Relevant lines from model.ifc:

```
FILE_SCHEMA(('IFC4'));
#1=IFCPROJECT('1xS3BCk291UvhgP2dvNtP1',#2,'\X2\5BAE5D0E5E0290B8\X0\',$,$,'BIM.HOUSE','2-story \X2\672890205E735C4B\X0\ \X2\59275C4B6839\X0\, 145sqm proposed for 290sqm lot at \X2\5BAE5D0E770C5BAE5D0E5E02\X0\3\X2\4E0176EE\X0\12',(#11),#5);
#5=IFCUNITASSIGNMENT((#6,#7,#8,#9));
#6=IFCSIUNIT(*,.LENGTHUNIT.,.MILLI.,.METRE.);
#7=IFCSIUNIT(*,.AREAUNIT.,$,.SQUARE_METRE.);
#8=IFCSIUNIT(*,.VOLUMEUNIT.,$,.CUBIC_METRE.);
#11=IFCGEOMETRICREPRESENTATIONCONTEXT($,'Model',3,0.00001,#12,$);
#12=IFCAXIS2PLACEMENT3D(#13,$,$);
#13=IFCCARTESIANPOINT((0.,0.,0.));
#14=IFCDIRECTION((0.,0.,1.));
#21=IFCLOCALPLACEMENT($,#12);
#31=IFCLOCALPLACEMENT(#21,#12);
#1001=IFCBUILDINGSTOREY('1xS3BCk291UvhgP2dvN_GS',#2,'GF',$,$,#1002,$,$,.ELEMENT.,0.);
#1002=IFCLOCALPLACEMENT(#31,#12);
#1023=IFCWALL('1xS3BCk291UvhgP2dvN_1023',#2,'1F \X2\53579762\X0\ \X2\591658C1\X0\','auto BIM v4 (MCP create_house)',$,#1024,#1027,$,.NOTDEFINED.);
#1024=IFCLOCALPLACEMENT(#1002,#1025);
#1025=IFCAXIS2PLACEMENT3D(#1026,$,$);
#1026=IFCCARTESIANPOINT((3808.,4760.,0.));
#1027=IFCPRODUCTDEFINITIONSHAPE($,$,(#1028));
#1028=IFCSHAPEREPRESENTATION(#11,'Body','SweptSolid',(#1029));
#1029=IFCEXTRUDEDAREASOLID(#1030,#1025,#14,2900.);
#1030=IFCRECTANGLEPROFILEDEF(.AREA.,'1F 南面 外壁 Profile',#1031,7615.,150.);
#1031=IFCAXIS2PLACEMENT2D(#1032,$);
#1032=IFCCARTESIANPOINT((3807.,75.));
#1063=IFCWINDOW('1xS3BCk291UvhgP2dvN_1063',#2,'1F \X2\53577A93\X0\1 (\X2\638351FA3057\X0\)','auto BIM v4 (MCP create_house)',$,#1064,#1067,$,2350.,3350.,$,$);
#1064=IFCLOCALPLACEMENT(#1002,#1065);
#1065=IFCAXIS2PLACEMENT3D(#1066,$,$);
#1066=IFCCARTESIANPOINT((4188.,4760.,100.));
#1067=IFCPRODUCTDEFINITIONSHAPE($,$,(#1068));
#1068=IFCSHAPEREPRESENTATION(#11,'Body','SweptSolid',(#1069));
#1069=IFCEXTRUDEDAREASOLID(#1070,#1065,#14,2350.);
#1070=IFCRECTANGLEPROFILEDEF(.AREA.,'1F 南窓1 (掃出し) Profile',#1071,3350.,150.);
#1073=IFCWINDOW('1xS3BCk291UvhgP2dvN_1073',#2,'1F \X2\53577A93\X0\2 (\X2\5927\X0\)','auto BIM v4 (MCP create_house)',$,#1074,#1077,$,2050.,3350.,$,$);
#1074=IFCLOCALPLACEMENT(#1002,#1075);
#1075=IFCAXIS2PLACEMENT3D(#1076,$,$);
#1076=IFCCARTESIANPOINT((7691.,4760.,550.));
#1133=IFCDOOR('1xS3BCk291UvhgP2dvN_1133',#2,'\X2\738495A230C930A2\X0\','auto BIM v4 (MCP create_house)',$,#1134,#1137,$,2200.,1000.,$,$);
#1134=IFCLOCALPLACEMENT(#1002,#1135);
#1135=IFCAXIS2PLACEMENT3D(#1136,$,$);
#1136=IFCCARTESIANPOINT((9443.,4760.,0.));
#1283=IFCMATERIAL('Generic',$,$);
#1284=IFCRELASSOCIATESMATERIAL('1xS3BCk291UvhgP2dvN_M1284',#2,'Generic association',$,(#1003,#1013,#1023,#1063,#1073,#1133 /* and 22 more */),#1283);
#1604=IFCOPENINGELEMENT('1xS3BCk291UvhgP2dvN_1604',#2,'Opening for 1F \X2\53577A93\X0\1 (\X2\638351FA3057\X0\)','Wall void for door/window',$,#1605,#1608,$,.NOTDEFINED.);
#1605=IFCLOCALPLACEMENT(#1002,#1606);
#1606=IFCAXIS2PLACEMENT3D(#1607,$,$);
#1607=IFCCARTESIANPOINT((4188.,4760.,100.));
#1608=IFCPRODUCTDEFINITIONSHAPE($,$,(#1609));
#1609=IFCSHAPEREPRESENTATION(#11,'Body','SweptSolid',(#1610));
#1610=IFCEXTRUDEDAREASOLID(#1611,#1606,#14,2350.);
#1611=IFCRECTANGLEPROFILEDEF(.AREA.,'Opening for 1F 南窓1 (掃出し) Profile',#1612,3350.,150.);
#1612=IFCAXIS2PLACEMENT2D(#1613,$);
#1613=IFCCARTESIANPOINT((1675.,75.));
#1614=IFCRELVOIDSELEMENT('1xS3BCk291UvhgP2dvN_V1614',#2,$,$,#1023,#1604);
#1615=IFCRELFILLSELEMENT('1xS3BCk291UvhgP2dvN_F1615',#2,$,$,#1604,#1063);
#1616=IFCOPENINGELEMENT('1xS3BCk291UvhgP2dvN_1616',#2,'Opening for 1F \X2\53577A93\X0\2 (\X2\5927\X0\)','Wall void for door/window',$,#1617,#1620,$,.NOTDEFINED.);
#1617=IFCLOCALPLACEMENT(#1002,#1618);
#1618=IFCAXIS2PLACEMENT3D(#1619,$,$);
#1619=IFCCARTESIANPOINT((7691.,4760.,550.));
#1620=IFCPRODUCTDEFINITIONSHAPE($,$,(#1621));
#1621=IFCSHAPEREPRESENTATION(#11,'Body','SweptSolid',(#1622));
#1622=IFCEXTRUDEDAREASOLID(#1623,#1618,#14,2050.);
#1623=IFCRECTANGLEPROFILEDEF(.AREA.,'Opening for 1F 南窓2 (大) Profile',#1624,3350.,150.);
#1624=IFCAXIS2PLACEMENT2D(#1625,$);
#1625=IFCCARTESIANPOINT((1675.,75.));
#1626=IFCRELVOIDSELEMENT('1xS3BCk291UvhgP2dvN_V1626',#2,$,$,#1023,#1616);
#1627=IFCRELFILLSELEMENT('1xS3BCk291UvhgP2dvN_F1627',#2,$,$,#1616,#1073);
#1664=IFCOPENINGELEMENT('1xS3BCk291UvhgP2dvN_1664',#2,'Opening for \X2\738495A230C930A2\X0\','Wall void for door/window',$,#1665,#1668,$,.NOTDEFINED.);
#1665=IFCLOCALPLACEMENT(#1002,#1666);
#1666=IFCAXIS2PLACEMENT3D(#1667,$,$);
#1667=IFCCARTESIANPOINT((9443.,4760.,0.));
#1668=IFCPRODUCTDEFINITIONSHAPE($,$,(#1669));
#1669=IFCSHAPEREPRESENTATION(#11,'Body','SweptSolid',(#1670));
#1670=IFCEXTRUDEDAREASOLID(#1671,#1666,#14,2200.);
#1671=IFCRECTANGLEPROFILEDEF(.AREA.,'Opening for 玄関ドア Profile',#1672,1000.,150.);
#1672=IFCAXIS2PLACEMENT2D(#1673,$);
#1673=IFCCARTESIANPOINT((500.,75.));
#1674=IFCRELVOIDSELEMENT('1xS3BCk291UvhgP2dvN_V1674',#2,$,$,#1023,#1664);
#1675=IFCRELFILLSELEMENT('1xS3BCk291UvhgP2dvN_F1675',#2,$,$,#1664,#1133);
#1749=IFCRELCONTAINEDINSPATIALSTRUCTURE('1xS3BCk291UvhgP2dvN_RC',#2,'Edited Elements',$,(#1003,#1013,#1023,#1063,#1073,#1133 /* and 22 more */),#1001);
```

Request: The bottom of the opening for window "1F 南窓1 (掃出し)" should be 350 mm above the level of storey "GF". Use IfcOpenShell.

```python
import numpy as np
import ifcopenshell
import ifcopenshell.api.geometry
import ifcopenshell.geom
import ifcopenshell.util.element
import ifcopenshell.util.placement
import ifcopenshell.util.shape
import ifcopenshell.util.unit

model = ifcopenshell.open("model.ifc")
unit_scale = ifcopenshell.util.unit.calculate_unit_scale(model)

window = model.by_id(1063)
opening = window.FillsVoids[0].RelatingOpeningElement
storey = ifcopenshell.util.element.get_container(window, ifc_class="IfcBuildingStorey")
level = ifcopenshell.util.placement.get_local_placement(storey.ObjectPlacement)[2, 3]

# The opening's origin need not be at the sill, so measure its lowest point.
shape = ifcopenshell.geom.create_shape(ifcopenshell.geom.settings(), opening)
bottom = ifcopenshell.util.shape.get_shape_bottom_elevation(shape, shape.geometry) / unit_scale
dz = level + 0.35 / unit_scale - bottom

shift = np.array([0.0, 0.0, dz])
# The window is not placed relative to its opening, so move both.
for product in (opening, window):
    matrix = ifcopenshell.util.placement.get_local_placement(product.ObjectPlacement)
    matrix[:3, 3] += shift
    ifcopenshell.api.geometry.edit_object_placement(model, product=product, matrix=matrix, is_si=False)

print(f"moved by {dz * unit_scale:+.3f} m")

model.write("model_updated.ifc")
```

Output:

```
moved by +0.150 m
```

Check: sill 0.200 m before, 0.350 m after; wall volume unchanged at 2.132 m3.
